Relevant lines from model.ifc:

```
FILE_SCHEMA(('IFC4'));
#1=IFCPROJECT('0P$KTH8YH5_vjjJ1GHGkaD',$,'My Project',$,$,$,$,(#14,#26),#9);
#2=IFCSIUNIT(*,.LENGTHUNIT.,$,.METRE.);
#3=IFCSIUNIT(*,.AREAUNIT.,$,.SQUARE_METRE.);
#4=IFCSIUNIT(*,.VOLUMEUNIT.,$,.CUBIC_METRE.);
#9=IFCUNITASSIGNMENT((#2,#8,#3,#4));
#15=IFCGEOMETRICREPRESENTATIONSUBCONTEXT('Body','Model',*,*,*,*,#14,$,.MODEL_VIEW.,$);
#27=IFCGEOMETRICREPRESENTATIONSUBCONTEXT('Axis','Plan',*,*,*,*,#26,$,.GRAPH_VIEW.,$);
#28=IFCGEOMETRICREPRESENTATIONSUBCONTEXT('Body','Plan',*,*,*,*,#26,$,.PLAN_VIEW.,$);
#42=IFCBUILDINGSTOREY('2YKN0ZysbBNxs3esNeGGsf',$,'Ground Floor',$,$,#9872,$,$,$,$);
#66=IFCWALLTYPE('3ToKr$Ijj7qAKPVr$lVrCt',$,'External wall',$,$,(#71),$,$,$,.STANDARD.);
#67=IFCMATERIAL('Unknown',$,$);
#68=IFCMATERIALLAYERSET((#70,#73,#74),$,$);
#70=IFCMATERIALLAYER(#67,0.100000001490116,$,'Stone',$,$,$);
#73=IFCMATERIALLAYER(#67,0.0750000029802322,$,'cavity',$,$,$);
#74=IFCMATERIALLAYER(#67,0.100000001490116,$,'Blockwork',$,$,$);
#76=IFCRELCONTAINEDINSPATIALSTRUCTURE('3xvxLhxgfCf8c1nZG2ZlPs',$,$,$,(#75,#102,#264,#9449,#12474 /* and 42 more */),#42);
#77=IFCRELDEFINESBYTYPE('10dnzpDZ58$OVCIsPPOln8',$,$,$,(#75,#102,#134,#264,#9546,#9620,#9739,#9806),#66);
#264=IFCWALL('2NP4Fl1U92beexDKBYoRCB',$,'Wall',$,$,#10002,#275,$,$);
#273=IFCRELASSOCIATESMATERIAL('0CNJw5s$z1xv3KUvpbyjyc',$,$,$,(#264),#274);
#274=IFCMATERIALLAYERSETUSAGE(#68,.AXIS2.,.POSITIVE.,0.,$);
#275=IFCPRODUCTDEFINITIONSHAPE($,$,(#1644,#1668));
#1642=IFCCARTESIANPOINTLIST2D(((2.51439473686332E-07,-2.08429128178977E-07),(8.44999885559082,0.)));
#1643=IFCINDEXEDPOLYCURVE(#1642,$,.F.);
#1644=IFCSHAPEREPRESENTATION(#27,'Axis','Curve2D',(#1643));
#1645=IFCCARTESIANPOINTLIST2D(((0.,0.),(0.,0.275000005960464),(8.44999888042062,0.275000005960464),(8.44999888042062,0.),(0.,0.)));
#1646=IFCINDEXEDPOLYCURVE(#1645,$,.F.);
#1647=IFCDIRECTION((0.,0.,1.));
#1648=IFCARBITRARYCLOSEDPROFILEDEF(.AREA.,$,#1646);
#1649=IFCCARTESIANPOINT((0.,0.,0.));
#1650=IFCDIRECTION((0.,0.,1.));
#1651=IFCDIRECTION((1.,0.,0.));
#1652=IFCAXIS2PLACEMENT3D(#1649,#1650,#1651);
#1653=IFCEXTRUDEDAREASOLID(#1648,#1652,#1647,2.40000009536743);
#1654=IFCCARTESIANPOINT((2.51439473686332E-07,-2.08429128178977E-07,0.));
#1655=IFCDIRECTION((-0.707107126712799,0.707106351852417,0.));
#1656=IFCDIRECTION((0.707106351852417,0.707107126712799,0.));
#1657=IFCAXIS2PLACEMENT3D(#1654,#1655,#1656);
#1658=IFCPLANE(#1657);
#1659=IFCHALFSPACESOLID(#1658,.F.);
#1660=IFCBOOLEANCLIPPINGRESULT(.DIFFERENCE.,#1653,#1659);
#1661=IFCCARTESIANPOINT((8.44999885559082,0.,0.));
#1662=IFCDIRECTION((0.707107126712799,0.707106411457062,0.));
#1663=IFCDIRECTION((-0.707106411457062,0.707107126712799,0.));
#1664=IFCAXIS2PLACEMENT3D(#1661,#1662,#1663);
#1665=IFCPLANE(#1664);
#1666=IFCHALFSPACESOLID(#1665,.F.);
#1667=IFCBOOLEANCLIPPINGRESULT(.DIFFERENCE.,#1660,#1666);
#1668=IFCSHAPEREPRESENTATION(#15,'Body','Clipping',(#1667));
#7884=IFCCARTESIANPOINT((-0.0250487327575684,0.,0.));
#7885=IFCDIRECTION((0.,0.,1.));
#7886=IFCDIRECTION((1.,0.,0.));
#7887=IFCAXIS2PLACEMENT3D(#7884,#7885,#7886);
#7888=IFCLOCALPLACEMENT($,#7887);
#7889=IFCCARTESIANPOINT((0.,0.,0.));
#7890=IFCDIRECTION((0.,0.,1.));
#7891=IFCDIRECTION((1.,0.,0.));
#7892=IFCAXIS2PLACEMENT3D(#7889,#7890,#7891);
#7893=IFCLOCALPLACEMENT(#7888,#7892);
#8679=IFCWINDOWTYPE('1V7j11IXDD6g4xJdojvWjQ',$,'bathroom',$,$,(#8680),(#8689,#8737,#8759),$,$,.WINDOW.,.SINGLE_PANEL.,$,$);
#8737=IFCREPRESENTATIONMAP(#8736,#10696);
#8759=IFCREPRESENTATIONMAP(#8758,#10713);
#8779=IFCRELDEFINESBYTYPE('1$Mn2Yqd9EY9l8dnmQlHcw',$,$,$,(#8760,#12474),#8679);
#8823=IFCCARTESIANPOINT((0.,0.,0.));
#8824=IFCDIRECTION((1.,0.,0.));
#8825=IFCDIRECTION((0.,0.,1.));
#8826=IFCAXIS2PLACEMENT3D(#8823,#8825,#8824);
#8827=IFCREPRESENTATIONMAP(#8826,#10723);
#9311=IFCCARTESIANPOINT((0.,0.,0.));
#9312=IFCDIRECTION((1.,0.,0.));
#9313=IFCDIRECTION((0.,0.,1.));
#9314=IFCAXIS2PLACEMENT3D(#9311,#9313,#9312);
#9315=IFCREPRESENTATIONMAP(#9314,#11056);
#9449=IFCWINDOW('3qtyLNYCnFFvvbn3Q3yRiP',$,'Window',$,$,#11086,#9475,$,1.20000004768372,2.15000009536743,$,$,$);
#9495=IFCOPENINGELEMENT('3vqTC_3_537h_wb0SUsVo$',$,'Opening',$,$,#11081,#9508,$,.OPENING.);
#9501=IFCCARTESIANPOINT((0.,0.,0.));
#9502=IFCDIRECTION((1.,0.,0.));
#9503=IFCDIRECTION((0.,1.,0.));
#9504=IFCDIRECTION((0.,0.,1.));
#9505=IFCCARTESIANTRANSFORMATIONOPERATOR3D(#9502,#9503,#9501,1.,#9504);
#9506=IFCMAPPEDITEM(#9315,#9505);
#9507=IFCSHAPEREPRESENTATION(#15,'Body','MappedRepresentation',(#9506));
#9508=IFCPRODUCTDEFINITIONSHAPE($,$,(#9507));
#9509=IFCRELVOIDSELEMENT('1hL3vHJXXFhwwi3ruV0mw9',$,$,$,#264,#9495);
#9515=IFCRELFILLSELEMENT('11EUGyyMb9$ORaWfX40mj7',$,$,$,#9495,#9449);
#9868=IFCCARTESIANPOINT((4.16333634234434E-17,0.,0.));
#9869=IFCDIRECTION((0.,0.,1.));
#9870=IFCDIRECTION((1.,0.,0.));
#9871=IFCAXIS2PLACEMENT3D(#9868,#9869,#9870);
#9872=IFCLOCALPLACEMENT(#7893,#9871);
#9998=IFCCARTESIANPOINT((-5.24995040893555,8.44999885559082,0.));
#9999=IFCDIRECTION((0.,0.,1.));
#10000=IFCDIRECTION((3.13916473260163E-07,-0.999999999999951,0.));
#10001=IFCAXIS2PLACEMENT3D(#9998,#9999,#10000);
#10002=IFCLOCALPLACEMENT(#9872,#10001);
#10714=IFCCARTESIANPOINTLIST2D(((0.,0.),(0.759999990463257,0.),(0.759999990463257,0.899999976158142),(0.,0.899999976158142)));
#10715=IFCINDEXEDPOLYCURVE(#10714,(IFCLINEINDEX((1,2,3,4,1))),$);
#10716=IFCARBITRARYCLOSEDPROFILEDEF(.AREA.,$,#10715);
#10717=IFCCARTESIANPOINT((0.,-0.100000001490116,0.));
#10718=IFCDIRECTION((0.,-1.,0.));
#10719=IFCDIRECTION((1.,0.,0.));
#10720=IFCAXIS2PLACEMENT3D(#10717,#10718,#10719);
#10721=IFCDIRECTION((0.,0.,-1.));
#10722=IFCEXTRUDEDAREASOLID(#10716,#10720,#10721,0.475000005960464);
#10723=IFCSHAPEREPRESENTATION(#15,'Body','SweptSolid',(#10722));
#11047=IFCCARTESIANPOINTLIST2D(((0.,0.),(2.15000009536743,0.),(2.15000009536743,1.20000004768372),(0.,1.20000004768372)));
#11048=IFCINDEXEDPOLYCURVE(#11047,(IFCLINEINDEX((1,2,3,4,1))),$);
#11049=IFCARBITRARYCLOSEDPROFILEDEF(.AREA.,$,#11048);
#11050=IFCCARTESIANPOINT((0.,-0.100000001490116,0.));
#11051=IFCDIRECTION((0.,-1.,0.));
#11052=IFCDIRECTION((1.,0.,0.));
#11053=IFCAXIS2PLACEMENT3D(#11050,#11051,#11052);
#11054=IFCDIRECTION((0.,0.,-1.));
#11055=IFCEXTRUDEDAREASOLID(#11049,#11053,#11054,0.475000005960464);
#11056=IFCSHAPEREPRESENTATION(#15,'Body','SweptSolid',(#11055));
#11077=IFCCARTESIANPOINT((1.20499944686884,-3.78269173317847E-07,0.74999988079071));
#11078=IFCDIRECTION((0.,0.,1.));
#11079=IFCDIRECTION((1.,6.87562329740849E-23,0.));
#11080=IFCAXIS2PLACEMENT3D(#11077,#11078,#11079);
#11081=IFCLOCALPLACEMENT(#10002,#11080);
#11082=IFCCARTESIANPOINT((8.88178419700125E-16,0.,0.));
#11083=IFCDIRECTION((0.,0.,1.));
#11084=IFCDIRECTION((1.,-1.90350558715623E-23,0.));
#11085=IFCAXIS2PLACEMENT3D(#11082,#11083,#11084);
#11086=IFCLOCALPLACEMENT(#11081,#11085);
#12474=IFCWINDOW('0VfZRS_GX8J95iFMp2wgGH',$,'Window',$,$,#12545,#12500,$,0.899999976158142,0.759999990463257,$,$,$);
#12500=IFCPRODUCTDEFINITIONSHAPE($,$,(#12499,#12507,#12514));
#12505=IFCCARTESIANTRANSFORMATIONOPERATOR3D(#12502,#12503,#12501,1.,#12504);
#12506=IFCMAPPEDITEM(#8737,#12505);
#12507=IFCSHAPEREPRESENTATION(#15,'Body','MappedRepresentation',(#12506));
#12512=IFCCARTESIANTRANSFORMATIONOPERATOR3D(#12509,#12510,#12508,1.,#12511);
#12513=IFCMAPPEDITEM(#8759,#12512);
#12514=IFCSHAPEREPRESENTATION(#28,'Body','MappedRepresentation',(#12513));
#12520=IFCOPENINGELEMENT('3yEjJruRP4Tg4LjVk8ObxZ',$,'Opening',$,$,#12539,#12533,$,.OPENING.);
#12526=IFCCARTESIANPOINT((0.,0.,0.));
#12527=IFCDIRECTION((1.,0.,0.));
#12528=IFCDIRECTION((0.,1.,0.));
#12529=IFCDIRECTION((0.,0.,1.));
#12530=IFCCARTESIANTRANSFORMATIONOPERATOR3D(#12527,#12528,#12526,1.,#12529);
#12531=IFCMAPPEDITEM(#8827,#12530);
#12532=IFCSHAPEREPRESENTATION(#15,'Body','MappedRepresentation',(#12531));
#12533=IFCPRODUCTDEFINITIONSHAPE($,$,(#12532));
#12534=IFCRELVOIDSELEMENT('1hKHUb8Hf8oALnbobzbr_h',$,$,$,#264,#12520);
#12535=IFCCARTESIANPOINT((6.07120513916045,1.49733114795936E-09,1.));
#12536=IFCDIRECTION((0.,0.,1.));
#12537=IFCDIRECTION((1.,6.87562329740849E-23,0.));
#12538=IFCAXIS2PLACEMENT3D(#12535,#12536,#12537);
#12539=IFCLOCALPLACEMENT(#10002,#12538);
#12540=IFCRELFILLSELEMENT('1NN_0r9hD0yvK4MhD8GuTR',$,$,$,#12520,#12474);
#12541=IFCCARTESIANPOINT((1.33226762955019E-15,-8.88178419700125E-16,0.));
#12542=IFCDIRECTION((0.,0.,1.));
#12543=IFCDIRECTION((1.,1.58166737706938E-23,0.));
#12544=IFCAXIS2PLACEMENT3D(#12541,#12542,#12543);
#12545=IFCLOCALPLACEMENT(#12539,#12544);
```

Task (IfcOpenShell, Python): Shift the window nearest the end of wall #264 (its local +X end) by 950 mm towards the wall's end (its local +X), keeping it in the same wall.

```python
import ifcopenshell
import ifcopenshell.api.geometry
import ifcopenshell.util.placement

model = ifcopenshell.open("model.ifc")

window = model.by_guid("0VfZRS_GX8J95iFMp2wgGH")
opening = window.FillsVoids[0].RelatingOpeningElement
wall = opening.VoidsElements[0].RelatingBuildingElement

wall_matrix = ifcopenshell.util.placement.get_local_placement(wall.ObjectPlacement)
shift = wall_matrix[:3, 0] * 0.95
before = ifcopenshell.util.placement.get_local_placement(window.ObjectPlacement)[:3, 3].copy()

# The window is placed relative to its opening, so it follows when the opening moves.
matrix = ifcopenshell.util.placement.get_local_placement(opening.ObjectPlacement)
matrix[:3, 3] += shift
ifcopenshell.api.geometry.edit_object_placement(
    model, product=opening, matrix=matrix, is_si=False, should_transform_children=True
)

after = ifcopenshell.util.placement.get_local_placement(window.ObjectPlacement)[:3, 3]
print("window moved by", (after - before).round(3) + 0.0)

model.write("model-out.ifc")
```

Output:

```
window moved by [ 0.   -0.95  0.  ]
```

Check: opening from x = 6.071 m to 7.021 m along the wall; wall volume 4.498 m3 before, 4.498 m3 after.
